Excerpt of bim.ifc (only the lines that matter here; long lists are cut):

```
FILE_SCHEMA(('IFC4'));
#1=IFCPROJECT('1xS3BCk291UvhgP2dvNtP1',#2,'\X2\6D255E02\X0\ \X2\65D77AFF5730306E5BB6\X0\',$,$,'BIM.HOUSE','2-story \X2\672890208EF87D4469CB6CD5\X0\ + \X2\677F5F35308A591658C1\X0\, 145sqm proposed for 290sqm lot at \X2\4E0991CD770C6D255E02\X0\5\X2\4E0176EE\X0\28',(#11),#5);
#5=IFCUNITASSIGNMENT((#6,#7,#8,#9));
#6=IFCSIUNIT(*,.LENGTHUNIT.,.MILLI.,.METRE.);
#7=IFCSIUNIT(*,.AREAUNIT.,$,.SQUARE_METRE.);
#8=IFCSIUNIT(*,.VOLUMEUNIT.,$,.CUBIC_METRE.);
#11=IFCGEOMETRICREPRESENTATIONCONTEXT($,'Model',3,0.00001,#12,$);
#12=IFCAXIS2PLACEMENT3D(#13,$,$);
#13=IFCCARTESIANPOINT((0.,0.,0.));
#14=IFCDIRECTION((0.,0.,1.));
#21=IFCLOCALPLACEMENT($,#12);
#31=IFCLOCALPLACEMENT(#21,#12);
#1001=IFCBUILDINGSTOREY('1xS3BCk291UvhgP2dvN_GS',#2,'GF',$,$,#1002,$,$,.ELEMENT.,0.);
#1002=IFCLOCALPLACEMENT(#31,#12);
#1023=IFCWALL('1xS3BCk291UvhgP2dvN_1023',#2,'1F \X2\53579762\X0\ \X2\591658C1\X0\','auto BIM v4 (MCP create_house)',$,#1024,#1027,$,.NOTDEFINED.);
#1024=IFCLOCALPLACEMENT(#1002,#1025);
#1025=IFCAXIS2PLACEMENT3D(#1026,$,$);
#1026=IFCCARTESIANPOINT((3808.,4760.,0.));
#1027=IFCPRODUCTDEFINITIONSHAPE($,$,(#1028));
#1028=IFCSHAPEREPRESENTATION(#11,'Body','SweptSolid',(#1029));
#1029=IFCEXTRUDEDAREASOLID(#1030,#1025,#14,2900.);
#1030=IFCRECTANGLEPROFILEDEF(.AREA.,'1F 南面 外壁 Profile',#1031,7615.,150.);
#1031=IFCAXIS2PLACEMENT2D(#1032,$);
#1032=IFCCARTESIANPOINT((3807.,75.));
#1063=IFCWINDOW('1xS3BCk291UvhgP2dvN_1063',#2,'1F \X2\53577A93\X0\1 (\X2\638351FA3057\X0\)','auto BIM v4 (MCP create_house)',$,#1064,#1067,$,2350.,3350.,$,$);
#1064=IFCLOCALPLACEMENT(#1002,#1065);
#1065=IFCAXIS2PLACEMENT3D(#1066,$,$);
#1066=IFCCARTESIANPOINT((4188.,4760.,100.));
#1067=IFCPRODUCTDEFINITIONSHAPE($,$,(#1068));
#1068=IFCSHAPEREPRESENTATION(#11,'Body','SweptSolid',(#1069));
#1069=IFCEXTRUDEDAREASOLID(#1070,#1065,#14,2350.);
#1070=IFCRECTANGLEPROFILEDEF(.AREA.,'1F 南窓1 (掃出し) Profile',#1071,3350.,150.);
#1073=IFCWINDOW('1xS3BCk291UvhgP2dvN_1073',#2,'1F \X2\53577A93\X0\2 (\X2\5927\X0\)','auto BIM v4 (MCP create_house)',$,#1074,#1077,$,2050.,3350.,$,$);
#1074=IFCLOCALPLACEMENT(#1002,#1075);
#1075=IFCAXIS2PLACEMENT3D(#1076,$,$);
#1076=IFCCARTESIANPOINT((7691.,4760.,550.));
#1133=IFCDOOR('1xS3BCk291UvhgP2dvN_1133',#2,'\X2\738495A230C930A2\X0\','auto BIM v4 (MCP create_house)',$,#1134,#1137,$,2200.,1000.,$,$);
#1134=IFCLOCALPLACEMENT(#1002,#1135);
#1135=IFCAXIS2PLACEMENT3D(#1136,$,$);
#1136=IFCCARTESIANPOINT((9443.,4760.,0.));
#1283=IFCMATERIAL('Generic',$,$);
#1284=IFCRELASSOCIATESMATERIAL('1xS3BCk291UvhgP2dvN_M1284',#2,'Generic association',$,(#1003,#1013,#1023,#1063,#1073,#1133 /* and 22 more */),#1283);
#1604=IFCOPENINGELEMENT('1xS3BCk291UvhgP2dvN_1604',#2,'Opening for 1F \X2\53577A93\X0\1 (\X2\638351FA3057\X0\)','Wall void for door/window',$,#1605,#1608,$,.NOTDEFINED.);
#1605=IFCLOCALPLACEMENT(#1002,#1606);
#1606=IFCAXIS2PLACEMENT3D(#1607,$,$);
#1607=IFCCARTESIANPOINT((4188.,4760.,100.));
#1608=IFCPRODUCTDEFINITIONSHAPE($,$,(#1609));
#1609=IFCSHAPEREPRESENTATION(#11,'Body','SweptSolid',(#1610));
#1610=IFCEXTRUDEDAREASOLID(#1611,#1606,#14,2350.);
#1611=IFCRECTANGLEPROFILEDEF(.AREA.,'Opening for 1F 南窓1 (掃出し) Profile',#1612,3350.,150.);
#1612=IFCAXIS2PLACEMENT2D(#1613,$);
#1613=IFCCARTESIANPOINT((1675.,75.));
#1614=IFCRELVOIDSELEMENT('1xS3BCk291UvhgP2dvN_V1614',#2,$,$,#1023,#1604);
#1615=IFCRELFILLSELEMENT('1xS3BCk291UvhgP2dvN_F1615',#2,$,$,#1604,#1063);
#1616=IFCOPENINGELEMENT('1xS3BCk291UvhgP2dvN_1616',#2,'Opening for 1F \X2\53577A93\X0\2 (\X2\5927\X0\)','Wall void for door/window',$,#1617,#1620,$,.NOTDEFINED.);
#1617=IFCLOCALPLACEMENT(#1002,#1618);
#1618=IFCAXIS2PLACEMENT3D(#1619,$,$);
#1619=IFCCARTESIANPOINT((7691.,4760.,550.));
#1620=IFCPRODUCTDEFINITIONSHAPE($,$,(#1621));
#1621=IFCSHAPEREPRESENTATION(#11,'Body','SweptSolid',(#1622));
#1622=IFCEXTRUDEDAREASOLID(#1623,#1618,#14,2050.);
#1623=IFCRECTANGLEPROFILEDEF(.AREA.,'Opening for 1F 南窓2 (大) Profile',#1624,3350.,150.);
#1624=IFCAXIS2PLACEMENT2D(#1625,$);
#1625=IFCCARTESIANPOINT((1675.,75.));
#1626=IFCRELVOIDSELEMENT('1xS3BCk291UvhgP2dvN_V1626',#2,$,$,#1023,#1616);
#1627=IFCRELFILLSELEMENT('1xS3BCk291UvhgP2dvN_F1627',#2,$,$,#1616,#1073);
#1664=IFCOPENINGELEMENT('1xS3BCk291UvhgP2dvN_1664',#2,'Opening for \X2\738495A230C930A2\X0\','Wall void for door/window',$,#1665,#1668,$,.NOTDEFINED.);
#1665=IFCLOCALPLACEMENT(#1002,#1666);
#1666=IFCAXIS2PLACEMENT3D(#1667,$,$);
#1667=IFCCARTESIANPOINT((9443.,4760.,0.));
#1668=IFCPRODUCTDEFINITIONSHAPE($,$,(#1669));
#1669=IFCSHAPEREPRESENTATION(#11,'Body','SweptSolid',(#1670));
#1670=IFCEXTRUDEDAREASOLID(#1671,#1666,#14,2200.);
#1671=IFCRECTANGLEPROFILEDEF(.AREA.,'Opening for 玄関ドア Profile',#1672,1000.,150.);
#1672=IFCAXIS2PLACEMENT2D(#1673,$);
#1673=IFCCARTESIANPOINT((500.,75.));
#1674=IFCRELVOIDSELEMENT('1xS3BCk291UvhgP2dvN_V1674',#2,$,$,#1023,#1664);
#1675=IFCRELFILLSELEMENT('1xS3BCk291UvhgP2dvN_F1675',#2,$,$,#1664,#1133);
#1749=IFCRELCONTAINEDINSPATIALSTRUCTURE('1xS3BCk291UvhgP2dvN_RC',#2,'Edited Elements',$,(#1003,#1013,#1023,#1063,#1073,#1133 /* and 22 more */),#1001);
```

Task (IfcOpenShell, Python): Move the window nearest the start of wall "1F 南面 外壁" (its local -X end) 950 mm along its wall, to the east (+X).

```python
import ifcopenshell
import ifcopenshell.api.geometry
import ifcopenshell.util.placement

model = ifcopenshell.open("bim.ifc")

window = model.by_guid("1xS3BCk291UvhgP2dvN_1063")
opening = window.FillsVoids[0].RelatingOpeningElement
wall = opening.VoidsElements[0].RelatingBuildingElement

wall_matrix = ifcopenshell.util.placement.get_local_placement(wall.ObjectPlacement)
shift = wall_matrix[:3, 0] * 950.0
before = ifcopenshell.util.placement.get_local_placement(window.ObjectPlacement)[:3, 3].copy()

# The window is not placed relative to its opening, so move both.
for product in (opening, window):
    matrix = ifcopenshell.util.placement.get_local_placement(product.ObjectPlacement)
    matrix[:3, 3] += shift
    ifcopenshell.api.geometry.edit_object_placement(model, product=product, matrix=matrix, is_si=False)

after = ifcopenshell.util.placement.get_local_placement(window.ObjectPlacement)[:3, 3]
print("window moved by", (after - before).round(3) + 0.0)

model.write("bim_updated.ifc")
```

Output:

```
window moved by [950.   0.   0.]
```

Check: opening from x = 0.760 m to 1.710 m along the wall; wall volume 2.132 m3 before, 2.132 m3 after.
